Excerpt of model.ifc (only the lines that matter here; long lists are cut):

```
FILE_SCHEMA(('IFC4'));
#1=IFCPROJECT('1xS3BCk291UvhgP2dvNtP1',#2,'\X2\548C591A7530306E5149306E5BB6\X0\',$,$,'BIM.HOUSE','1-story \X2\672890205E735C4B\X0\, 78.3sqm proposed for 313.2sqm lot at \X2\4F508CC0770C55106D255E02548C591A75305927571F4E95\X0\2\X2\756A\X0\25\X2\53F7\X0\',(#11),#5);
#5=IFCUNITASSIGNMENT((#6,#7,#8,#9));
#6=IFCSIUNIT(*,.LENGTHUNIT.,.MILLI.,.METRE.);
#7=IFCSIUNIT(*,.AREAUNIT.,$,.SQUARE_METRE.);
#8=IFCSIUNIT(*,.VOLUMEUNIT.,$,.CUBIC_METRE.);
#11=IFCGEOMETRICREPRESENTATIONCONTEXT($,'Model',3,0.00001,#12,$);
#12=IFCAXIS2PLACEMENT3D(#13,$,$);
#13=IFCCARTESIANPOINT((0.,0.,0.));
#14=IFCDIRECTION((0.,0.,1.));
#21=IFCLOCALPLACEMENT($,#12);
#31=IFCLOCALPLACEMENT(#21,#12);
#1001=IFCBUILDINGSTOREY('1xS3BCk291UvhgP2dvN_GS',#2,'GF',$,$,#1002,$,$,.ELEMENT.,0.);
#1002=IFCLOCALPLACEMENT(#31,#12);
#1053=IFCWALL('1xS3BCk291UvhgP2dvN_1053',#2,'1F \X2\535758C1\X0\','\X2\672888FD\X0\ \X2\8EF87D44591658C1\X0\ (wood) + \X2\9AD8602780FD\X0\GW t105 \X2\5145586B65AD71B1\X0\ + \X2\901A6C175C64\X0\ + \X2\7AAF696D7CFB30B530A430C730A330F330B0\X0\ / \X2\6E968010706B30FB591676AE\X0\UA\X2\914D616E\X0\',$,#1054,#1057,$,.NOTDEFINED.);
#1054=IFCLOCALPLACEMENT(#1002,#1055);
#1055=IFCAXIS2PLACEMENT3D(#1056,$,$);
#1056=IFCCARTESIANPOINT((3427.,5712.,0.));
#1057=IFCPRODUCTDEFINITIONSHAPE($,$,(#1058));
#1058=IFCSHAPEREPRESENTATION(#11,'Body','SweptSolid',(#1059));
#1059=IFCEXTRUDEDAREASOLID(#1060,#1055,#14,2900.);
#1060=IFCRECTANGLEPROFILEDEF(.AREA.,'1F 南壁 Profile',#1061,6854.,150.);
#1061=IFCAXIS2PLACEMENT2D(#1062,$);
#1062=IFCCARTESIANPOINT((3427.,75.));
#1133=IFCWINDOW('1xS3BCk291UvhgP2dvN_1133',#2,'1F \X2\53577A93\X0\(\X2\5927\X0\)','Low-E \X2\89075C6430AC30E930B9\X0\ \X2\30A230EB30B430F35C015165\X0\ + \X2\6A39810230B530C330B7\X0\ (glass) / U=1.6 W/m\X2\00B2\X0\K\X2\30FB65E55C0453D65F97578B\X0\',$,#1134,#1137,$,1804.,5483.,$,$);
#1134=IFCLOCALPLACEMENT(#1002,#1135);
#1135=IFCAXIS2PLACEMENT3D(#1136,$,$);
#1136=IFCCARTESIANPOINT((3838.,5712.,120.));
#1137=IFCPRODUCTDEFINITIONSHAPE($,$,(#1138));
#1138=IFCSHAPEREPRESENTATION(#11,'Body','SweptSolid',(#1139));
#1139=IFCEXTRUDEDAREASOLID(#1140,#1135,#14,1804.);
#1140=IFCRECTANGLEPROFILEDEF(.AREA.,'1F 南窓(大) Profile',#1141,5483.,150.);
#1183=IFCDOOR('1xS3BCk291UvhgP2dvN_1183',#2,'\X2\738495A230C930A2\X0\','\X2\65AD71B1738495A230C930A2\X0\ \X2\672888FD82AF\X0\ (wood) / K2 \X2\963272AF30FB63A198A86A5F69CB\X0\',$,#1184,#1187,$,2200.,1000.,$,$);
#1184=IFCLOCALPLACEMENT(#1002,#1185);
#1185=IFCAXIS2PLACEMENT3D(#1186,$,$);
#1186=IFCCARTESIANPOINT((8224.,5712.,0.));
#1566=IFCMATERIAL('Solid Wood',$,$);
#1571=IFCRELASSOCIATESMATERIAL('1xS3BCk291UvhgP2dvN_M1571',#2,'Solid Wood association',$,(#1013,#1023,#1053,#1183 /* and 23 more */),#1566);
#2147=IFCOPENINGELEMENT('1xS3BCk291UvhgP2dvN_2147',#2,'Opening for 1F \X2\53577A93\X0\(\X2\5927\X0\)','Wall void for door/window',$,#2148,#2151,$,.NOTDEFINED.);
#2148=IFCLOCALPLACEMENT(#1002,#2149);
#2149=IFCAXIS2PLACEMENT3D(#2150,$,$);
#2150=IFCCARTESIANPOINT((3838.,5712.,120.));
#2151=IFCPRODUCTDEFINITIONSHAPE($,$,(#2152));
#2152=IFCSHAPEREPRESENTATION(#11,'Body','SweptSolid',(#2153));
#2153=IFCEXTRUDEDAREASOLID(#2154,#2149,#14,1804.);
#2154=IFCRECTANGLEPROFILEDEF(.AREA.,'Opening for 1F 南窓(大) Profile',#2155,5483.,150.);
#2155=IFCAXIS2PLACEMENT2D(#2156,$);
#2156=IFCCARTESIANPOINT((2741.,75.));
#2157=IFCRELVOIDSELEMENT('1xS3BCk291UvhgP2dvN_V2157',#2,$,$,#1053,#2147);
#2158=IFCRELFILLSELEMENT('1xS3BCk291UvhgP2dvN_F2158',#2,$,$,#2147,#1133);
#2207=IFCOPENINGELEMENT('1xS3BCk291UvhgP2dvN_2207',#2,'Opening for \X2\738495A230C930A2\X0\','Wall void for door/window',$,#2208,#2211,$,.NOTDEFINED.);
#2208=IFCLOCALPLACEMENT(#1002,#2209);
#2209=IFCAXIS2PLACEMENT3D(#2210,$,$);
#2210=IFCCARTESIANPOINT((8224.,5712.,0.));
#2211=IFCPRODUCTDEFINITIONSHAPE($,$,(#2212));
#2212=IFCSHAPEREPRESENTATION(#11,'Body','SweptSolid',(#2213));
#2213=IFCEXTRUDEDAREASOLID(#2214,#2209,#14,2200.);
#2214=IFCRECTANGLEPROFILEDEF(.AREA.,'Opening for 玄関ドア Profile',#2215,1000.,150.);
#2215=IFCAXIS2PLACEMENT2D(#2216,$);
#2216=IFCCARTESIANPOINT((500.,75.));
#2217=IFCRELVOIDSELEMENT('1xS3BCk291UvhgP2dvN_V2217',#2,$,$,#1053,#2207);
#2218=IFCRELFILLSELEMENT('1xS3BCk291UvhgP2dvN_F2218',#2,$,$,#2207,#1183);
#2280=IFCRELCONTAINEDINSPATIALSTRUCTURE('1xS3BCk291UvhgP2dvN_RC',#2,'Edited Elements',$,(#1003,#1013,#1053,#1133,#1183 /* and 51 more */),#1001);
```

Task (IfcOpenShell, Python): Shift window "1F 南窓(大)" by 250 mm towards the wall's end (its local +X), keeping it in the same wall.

```python
import ifcopenshell
import ifcopenshell.api.geometry
import ifcopenshell.util.placement
import ifcopenshell.util.unit

model = ifcopenshell.open("model.ifc")
unit_scale = ifcopenshell.util.unit.calculate_unit_scale(model)

window = model.by_guid("1xS3BCk291UvhgP2dvN_1133")
opening = window.FillsVoids[0].RelatingOpeningElement
wall = opening.VoidsElements[0].RelatingBuildingElement

wall_matrix = ifcopenshell.util.placement.get_local_placement(wall.ObjectPlacement)
shift = wall_matrix[:3, 0] * 0.25 / unit_scale
before = ifcopenshell.util.placement.get_local_placement(window.ObjectPlacement)[:3, 3].copy()

# The window is not placed relative to its opening, so move both.
for product in (opening, window):
    matrix = ifcopenshell.util.placement.get_local_placement(product.ObjectPlacement)
    matrix[:3, 3] += shift
    ifcopenshell.api.geometry.edit_object_placement(model, product=product, matrix=matrix, is_si=False)

after = ifcopenshell.util.placement.get_local_placement(window.ObjectPlacement)[:3, 3]
print("window moved by", (after - before).round(3) + 0.0)

model.write("model_edited.ifc")
```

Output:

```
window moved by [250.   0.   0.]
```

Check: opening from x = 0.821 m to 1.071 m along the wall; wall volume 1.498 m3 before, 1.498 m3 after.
